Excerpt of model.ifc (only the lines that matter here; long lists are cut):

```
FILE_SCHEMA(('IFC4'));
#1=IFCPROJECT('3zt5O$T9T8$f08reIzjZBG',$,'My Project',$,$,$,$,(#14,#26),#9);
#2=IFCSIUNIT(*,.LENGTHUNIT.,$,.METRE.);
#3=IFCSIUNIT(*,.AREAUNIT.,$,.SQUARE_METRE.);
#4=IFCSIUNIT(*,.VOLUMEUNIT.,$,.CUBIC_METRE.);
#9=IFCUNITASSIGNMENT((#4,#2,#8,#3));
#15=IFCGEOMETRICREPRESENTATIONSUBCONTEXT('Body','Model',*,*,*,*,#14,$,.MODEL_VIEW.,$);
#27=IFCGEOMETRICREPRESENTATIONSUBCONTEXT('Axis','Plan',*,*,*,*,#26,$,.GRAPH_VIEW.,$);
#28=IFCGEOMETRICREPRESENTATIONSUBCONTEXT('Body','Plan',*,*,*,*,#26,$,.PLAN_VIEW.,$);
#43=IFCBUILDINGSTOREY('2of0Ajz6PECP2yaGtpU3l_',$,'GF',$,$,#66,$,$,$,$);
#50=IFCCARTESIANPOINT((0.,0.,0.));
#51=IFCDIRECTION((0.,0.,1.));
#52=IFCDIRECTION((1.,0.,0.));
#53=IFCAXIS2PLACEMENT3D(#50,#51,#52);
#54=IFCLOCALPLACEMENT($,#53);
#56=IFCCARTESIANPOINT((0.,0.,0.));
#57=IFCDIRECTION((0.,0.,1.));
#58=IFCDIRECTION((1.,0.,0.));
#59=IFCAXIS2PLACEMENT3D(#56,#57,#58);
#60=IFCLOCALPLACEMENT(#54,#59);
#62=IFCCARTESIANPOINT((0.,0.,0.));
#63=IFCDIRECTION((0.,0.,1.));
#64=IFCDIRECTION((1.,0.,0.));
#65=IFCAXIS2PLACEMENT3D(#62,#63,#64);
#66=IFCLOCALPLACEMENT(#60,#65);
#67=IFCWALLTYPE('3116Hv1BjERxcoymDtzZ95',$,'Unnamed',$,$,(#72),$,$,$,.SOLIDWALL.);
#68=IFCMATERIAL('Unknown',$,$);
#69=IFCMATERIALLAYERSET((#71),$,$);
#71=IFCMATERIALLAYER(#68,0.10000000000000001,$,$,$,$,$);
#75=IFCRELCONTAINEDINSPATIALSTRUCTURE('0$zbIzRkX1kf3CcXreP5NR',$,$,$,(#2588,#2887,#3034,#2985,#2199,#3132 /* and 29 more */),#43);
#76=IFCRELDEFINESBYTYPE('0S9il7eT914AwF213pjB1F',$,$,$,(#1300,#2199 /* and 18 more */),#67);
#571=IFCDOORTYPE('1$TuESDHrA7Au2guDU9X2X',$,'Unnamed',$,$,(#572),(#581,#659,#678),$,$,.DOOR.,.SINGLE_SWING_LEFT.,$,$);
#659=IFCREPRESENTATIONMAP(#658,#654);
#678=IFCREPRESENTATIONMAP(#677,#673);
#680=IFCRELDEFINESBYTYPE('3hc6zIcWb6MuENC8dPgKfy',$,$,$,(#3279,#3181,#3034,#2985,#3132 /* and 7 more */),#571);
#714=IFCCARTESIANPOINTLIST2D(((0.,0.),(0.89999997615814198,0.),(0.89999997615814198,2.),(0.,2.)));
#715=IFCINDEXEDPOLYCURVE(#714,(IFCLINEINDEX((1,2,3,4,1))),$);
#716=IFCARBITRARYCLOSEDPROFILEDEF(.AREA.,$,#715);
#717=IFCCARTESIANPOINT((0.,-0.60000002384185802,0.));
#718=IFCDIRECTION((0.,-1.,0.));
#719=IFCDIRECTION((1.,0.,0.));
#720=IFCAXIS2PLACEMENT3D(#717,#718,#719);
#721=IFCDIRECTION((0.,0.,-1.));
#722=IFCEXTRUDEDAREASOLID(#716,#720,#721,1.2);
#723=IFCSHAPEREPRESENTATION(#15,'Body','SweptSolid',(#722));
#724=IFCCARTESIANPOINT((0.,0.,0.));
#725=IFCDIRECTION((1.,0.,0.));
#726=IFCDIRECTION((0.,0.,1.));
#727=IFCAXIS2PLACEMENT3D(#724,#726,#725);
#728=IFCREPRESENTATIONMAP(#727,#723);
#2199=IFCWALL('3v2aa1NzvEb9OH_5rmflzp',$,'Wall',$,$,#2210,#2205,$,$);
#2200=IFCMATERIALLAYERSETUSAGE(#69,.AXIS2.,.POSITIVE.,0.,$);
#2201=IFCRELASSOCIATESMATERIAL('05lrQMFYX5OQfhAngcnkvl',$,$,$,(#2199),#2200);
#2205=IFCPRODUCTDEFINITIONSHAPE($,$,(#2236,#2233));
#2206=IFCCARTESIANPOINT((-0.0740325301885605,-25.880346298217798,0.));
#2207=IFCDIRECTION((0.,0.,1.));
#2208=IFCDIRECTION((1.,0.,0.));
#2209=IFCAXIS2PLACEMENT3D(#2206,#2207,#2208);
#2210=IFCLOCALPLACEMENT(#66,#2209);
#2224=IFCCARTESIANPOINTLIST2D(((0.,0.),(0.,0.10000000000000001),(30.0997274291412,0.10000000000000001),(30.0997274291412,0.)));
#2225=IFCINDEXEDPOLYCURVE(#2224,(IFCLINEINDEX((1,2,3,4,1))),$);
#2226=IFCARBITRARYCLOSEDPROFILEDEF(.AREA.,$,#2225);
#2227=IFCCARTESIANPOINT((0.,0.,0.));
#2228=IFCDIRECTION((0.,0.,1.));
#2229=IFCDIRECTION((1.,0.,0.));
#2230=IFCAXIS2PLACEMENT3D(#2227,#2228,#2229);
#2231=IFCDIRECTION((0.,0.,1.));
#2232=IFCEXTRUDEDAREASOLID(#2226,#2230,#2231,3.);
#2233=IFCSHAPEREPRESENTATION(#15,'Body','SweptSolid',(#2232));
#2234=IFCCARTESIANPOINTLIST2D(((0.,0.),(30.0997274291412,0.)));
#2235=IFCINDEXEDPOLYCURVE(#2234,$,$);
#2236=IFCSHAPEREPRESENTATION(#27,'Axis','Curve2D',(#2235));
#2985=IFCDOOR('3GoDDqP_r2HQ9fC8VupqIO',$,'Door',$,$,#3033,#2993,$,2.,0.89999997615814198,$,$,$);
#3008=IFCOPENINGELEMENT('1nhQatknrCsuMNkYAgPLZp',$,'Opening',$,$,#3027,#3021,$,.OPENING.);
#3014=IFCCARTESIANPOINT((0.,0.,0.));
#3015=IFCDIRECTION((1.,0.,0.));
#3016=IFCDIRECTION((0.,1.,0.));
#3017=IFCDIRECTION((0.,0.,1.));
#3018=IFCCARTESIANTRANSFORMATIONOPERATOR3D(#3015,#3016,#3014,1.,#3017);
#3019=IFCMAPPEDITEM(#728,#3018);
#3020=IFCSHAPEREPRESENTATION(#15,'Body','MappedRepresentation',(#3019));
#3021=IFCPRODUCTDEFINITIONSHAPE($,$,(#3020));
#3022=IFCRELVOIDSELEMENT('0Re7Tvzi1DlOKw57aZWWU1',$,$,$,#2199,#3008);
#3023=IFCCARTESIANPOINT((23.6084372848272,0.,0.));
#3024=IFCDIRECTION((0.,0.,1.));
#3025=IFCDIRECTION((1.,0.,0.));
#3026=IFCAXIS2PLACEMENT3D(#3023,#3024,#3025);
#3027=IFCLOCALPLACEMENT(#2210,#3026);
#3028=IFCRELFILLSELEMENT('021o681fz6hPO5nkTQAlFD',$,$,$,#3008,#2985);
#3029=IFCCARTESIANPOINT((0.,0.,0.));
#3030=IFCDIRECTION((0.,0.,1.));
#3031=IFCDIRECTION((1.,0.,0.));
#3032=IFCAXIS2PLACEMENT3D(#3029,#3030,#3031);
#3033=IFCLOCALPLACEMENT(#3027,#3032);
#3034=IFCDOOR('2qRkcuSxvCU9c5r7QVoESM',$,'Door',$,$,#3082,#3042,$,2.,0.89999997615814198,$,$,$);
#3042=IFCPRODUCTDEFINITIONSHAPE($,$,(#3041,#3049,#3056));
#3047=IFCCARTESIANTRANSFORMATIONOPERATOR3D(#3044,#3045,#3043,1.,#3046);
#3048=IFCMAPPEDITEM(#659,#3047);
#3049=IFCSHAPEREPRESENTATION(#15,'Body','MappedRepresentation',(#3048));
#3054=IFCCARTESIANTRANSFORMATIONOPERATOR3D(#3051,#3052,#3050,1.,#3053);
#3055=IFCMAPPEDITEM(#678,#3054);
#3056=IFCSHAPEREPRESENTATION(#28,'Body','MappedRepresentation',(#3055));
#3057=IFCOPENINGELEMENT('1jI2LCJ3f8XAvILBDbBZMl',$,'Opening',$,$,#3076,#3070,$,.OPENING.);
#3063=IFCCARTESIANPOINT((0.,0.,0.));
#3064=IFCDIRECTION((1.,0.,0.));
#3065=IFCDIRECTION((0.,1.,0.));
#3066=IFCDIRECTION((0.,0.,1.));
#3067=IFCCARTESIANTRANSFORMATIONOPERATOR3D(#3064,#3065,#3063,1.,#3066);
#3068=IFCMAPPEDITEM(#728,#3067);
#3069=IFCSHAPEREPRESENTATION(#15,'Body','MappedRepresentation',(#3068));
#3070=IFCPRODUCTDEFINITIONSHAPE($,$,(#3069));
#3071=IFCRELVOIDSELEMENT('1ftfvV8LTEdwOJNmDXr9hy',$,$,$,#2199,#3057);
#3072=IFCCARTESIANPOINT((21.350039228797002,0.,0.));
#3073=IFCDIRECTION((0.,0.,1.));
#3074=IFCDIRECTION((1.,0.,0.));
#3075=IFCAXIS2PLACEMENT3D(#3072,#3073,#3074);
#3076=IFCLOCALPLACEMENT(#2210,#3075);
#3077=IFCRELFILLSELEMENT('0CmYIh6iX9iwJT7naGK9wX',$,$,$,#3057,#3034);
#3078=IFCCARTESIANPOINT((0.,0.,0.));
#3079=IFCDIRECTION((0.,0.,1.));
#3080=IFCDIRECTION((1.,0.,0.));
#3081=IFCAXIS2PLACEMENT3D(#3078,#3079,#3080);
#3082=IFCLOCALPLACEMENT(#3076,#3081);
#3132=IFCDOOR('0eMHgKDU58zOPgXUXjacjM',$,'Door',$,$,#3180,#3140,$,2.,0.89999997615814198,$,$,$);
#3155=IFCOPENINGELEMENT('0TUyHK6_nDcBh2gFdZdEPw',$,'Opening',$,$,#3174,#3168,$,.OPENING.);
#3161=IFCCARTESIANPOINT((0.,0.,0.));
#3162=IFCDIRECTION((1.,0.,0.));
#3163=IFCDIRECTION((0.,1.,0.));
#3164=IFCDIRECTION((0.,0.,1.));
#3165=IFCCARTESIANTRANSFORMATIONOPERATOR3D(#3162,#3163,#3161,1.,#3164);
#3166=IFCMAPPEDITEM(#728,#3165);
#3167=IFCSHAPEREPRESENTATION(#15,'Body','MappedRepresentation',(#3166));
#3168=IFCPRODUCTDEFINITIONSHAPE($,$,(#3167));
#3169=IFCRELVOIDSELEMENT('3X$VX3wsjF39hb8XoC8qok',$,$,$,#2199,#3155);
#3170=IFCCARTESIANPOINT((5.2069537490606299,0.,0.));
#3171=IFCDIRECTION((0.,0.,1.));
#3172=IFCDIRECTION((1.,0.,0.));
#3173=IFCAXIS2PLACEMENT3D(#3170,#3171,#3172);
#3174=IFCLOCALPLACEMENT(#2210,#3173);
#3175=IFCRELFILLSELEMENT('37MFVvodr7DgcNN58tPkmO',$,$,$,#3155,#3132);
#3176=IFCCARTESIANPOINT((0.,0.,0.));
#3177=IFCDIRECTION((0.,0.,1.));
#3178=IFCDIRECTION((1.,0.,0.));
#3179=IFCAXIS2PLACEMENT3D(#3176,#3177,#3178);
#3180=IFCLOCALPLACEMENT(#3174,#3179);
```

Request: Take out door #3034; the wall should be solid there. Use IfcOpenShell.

```python
import ifcopenshell
import ifcopenshell.api.feature
import ifcopenshell.api.root
import ifcopenshell.geom
import ifcopenshell.util.shape

model = ifcopenshell.open("model.ifc")
settings = ifcopenshell.geom.settings()


def volume(element):
    """Net volume in cubic metres, openings subtracted."""
    shape = ifcopenshell.geom.create_shape(settings, element)
    return ifcopenshell.util.shape.get_volume(shape.geometry)


door = model.by_guid("2qRkcuSxvCU9c5r7QVoESM")
opening = door.FillsVoids[0].RelatingOpeningElement
wall = opening.VoidsElements[0].RelatingBuildingElement
before = volume(wall)

ifcopenshell.api.root.remove_product(model, product=door)
ifcopenshell.api.feature.remove_feature(model, feature=opening)

after = volume(wall)

print(f"wall volume {before:.3f} -> {after:.3f} m3")

model.write("model_updated.ifc")
```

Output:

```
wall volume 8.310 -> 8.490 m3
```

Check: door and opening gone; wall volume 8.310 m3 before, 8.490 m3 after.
